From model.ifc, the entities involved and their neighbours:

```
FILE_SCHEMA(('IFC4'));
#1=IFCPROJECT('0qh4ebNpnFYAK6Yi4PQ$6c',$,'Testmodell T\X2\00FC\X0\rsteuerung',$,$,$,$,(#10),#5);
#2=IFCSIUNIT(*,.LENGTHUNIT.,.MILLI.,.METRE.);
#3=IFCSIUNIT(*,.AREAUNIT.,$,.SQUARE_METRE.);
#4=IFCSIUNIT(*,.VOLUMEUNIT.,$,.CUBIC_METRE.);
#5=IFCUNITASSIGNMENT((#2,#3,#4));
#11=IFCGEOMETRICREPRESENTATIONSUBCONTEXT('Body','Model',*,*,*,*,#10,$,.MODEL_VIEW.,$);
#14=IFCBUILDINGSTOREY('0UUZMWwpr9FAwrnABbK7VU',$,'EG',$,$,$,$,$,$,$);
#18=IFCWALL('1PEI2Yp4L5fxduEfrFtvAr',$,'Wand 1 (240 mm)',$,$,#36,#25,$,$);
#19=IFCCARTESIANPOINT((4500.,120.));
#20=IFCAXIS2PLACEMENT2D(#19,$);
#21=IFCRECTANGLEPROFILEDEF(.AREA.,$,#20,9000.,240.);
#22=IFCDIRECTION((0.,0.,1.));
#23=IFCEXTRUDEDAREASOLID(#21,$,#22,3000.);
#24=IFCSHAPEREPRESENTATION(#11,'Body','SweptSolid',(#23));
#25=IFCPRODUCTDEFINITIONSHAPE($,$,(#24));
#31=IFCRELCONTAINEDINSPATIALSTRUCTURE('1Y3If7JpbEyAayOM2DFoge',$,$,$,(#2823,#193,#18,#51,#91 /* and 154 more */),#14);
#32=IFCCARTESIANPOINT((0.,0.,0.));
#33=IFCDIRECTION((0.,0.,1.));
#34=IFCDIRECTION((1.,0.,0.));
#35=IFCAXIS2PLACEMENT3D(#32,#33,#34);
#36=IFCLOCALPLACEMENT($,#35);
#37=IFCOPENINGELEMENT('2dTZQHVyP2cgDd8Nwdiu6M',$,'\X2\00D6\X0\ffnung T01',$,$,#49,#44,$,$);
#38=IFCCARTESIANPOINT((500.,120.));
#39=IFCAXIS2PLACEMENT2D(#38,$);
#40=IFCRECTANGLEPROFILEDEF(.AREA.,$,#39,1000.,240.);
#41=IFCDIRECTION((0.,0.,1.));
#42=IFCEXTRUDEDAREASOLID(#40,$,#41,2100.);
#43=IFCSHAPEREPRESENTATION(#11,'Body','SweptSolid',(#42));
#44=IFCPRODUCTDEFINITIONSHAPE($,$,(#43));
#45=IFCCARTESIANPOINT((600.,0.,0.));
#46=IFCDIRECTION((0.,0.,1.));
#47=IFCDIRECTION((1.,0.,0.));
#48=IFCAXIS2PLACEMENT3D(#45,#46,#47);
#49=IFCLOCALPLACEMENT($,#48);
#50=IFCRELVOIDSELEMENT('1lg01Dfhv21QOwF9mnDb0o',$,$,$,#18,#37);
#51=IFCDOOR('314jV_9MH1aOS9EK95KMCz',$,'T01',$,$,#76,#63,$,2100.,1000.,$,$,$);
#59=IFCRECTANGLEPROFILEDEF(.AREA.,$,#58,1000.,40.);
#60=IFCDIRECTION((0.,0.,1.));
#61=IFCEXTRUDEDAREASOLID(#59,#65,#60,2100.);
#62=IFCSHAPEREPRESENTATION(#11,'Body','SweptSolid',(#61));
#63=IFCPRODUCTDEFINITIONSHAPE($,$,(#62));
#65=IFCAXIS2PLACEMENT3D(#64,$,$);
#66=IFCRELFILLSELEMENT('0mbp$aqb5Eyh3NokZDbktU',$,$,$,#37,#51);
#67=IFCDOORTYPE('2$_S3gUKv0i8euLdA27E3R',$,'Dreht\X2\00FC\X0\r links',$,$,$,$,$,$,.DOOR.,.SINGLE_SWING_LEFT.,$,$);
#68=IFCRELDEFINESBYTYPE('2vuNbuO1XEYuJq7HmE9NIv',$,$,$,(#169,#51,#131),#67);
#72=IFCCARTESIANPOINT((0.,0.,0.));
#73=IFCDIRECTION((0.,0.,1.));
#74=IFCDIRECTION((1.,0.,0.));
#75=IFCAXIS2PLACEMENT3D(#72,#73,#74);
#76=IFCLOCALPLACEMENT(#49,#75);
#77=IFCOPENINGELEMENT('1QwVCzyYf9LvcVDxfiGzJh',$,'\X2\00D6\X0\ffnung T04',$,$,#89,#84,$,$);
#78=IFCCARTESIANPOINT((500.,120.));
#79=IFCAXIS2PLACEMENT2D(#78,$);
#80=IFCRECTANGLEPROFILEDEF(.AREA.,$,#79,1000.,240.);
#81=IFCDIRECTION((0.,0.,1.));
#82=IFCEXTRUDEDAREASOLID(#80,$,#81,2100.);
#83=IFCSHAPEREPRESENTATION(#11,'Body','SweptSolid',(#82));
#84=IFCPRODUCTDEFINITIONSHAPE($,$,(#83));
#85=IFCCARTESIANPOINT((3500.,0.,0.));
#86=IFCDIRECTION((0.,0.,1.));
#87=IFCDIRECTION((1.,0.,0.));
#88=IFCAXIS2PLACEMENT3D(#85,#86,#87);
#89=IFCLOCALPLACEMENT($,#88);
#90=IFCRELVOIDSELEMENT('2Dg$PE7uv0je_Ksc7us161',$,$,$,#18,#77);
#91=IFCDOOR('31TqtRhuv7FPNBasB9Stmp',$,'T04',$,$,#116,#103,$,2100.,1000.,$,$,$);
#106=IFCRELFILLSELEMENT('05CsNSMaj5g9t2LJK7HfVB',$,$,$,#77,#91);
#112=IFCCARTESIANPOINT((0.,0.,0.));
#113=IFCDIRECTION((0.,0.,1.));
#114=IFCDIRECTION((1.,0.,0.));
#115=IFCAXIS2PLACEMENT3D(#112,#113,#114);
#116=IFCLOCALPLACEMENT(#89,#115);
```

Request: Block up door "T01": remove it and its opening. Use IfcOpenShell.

```python
import ifcopenshell
import ifcopenshell.api.feature
import ifcopenshell.api.root
import ifcopenshell.geom
import ifcopenshell.util.shape

model = ifcopenshell.open("model.ifc")
settings = ifcopenshell.geom.settings()


def volume(element):
    """Net volume in cubic metres, openings subtracted."""
    shape = ifcopenshell.geom.create_shape(settings, element)
    return ifcopenshell.util.shape.get_volume(shape.geometry)


door = model.by_guid("314jV_9MH1aOS9EK95KMCz")
opening = door.FillsVoids[0].RelatingOpeningElement
wall = opening.VoidsElements[0].RelatingBuildingElement
before = volume(wall)

ifcopenshell.api.root.remove_product(model, product=door)
ifcopenshell.api.feature.remove_feature(model, feature=opening)

after = volume(wall)

print(f"wall volume {before:.3f} -> {after:.3f} m3")

model.write("model_v2.ifc")
```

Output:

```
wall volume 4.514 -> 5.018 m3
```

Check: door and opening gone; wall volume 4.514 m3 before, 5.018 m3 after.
